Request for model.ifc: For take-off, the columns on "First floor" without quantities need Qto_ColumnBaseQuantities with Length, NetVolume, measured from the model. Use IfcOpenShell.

First a look at what the model holds.

```python
import ifcopenshell
import ifcopenshell.util.element
import ifcopenshell.util.unit

model = ifcopenshell.open("model.ifc")
print(model.schema)
for unit_type in ("LENGTHUNIT", "AREAUNIT", "VOLUMEUNIT"):
    print(unit_type, ifcopenshell.util.unit.calculate_unit_scale(model, unit_type))
storey = next(s for s in model.by_type("IfcBuildingStorey") if s.Name == "First floor")
columns = [e for e in ifcopenshell.util.element.get_decomposition(storey) if e.is_a("IfcColumn")]
for e in sorted(columns, key=lambda e: e.id()):
    print(e.id(), e.is_a(), e.Name, list(ifcopenshell.util.element.get_psets(e, qtos_only=True)), sep=" | ")
```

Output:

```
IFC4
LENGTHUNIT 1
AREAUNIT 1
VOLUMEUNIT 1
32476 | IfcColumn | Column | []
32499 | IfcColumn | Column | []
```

```python
import ifcopenshell
import ifcopenshell.api.pset
import ifcopenshell.geom
import ifcopenshell.util.element
import ifcopenshell.util.shape
import ifcopenshell.util.unit

model = ifcopenshell.open("model.ifc")
unit_scale = ifcopenshell.util.unit.calculate_unit_scale(model)
volume_scale = ifcopenshell.util.unit.calculate_unit_scale(model, "VOLUMEUNIT")
settings = ifcopenshell.geom.settings()

storey = next(s for s in model.by_type("IfcBuildingStorey") if s.Name == "First floor")
columns = [e for e in ifcopenshell.util.element.get_decomposition(storey) if e.is_a("IfcColumn")]

for e in sorted(columns, key=lambda e: e.id()):
    if ifcopenshell.util.element.get_psets(e, qtos_only=True, should_inherit=False):
        continue
    # Geometry comes back in metres, in the element's own axes.
    shape = ifcopenshell.geom.create_shape(settings, e)
    values = {
        "Length": ifcopenshell.util.shape.get_z(shape.geometry) / unit_scale,
        "NetVolume": ifcopenshell.util.shape.get_volume(shape.geometry) / volume_scale,
    }
    qto = ifcopenshell.api.pset.add_qto(model, product=e, name="Qto_ColumnBaseQuantities")
    ifcopenshell.api.pset.edit_qto(model, qto=qto, properties=values)
    print(e.id(), {k: round(v, 3) for k, v in values.items()})

model.write("model_edited.ifc")
```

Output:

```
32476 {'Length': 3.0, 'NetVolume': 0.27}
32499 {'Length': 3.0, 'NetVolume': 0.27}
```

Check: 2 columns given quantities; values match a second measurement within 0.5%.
